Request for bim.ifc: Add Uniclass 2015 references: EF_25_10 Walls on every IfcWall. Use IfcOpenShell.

First a look at what the model holds.

```python
import ifcopenshell

model = ifcopenshell.open("bim.ifc")
print(model.schema)
print("classifications:", [c.Name for c in model.by_type("IfcClassification")])
for ifc_class in ("IfcDoor", "IfcRoof", "IfcStair", "IfcWall", "IfcWindow"):
    print(ifc_class, len(model.by_type(ifc_class)))
```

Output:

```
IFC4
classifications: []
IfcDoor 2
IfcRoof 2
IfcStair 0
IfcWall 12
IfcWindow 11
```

```python
import ifcopenshell
import ifcopenshell.api.classification

model = ifcopenshell.open("bim.ifc")

system = ifcopenshell.api.classification.add_classification(model, classification="Uniclass 2015")

codes = {
    "IfcWall": ("EF_25_10", "Walls"),
}
for ifc_class, (code, name) in codes.items():
    products = model.by_type(ifc_class)
    ifcopenshell.api.classification.add_reference(
        model, products=products, classification=system, identification=code, name=name
    )
    print(code, len(products))

model.write("bim_rev.ifc")
```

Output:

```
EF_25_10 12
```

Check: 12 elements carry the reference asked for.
